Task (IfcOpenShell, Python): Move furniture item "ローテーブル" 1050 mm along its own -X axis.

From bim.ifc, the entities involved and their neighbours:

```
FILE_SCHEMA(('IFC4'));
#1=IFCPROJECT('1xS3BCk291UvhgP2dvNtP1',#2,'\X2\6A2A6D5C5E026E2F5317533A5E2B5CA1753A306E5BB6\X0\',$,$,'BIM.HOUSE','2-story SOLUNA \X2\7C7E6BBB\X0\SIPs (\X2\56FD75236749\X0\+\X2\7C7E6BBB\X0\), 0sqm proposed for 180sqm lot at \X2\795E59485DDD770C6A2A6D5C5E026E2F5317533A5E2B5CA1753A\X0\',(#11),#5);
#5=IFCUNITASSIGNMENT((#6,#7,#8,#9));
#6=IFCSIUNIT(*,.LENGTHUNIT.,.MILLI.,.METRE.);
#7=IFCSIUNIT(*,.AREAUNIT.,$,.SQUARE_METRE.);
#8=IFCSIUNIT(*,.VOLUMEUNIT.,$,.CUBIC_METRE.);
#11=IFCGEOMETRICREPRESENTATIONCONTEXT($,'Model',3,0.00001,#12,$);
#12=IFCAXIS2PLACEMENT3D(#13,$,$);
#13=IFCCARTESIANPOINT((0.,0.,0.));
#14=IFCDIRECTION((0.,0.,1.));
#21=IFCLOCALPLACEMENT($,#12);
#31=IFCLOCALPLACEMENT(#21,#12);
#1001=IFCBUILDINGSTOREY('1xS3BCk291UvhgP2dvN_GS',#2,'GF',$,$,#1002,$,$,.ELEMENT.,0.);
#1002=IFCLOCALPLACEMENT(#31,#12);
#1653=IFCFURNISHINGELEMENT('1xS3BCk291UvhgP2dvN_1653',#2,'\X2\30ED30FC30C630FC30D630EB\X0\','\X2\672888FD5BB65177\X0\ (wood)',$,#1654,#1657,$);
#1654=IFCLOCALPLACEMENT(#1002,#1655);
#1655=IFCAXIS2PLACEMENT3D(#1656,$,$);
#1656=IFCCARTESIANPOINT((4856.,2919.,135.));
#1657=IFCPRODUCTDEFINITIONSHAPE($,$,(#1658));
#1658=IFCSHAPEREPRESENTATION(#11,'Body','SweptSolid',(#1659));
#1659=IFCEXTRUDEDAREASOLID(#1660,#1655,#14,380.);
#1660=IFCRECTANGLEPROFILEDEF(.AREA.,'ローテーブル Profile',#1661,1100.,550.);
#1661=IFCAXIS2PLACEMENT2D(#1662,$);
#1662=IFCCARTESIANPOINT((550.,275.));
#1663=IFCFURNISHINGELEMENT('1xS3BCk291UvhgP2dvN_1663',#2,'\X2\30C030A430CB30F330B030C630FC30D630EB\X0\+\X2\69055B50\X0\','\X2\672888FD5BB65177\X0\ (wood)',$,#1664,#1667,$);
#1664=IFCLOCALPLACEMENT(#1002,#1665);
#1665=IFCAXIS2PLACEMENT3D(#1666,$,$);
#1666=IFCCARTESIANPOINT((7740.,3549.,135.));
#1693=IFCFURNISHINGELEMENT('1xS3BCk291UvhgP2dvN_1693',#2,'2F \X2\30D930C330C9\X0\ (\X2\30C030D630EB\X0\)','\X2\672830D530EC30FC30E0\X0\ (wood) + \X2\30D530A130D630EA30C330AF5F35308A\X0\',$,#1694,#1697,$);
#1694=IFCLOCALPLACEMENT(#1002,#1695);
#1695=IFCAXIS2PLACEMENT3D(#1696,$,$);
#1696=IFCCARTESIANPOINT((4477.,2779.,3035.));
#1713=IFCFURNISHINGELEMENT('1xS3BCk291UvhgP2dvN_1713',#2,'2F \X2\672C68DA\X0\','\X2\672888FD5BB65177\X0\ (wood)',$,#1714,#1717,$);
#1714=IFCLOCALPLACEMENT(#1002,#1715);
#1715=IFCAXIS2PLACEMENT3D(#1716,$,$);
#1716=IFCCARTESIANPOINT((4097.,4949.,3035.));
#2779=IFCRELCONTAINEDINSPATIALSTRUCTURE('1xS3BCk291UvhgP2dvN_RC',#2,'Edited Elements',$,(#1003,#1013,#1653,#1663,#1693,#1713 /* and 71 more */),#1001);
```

```python
import ifcopenshell
import ifcopenshell.api.geometry
import ifcopenshell.util.placement

model = ifcopenshell.open("bim.ifc")

item = model.by_guid("1xS3BCk291UvhgP2dvN_1653")
matrix = ifcopenshell.util.placement.get_local_placement(item.ObjectPlacement)
matrix[:3, 3] -= matrix[:3, 0] * 1050.0
ifcopenshell.api.geometry.edit_object_placement(model, product=item, matrix=matrix, is_si=False)

print(ifcopenshell.util.placement.get_local_placement(item.ObjectPlacement).round(3) + 0.0)

model.write("bim_rev.ifc")
```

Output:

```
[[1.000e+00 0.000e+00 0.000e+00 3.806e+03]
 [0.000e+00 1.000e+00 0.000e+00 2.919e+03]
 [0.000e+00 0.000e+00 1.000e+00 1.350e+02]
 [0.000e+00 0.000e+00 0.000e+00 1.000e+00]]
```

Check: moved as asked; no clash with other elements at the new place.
